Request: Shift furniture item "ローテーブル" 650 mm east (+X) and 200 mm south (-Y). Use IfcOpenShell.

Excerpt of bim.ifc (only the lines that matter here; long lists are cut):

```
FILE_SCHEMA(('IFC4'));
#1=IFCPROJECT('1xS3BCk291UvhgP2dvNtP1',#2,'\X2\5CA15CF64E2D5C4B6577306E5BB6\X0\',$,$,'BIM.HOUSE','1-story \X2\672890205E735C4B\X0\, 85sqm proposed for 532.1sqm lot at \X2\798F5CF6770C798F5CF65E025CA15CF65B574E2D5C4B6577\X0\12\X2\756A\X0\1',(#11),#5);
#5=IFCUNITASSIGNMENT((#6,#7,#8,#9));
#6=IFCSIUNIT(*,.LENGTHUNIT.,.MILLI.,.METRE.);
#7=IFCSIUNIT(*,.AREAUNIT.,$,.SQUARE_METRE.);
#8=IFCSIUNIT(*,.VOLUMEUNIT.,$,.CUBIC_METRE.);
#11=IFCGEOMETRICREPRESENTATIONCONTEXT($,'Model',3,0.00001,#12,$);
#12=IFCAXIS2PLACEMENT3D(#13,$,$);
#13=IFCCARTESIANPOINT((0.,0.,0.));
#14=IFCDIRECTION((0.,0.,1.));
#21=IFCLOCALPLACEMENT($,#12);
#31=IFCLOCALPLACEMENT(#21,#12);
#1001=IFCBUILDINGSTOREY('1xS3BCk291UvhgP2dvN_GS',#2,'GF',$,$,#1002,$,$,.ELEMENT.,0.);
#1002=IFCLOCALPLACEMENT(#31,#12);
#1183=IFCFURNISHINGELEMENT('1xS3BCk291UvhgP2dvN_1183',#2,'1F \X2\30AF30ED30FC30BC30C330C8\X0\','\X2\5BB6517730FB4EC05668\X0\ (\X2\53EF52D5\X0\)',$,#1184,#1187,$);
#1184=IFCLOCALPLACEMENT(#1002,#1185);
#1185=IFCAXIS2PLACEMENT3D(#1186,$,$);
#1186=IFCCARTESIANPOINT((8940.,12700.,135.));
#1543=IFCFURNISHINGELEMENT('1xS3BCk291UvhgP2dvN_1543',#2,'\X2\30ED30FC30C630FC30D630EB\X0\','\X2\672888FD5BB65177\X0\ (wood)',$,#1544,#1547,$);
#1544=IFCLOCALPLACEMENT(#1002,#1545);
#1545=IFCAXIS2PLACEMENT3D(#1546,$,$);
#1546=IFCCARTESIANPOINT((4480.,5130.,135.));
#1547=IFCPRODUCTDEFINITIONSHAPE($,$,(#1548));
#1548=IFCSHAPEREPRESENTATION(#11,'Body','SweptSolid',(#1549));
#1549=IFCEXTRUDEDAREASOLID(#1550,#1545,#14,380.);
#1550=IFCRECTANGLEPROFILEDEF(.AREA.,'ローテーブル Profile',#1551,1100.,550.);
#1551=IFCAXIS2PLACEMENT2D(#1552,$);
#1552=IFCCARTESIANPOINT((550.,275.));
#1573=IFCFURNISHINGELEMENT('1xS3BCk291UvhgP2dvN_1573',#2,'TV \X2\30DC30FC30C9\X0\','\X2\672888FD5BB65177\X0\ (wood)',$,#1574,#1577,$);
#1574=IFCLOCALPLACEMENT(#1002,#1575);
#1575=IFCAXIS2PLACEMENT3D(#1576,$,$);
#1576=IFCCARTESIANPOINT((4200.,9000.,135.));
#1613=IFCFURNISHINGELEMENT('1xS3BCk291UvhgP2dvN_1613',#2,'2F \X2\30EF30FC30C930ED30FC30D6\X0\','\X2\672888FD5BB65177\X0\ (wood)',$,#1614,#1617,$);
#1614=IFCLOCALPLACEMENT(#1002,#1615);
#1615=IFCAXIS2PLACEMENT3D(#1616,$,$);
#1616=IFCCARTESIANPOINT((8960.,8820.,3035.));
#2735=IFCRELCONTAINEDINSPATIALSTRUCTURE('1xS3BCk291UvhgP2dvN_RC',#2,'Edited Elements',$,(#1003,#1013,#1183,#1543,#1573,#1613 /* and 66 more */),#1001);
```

```python
import ifcopenshell
import ifcopenshell.api.geometry
import ifcopenshell.util.placement

model = ifcopenshell.open("bim.ifc")

item = model.by_guid("1xS3BCk291UvhgP2dvN_1543")
matrix = ifcopenshell.util.placement.get_local_placement(item.ObjectPlacement)
matrix[0, 3] += 650.0
matrix[1, 3] -= 200.0
ifcopenshell.api.geometry.edit_object_placement(model, product=item, matrix=matrix, is_si=False)

print(ifcopenshell.util.placement.get_local_placement(item.ObjectPlacement).round(3) + 0.0)

model.write("bim_v2.ifc")
```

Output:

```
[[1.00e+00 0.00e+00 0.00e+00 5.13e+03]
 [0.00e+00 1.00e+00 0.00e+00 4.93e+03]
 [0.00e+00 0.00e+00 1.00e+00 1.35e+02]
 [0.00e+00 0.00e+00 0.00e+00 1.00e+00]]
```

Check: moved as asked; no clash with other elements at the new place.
